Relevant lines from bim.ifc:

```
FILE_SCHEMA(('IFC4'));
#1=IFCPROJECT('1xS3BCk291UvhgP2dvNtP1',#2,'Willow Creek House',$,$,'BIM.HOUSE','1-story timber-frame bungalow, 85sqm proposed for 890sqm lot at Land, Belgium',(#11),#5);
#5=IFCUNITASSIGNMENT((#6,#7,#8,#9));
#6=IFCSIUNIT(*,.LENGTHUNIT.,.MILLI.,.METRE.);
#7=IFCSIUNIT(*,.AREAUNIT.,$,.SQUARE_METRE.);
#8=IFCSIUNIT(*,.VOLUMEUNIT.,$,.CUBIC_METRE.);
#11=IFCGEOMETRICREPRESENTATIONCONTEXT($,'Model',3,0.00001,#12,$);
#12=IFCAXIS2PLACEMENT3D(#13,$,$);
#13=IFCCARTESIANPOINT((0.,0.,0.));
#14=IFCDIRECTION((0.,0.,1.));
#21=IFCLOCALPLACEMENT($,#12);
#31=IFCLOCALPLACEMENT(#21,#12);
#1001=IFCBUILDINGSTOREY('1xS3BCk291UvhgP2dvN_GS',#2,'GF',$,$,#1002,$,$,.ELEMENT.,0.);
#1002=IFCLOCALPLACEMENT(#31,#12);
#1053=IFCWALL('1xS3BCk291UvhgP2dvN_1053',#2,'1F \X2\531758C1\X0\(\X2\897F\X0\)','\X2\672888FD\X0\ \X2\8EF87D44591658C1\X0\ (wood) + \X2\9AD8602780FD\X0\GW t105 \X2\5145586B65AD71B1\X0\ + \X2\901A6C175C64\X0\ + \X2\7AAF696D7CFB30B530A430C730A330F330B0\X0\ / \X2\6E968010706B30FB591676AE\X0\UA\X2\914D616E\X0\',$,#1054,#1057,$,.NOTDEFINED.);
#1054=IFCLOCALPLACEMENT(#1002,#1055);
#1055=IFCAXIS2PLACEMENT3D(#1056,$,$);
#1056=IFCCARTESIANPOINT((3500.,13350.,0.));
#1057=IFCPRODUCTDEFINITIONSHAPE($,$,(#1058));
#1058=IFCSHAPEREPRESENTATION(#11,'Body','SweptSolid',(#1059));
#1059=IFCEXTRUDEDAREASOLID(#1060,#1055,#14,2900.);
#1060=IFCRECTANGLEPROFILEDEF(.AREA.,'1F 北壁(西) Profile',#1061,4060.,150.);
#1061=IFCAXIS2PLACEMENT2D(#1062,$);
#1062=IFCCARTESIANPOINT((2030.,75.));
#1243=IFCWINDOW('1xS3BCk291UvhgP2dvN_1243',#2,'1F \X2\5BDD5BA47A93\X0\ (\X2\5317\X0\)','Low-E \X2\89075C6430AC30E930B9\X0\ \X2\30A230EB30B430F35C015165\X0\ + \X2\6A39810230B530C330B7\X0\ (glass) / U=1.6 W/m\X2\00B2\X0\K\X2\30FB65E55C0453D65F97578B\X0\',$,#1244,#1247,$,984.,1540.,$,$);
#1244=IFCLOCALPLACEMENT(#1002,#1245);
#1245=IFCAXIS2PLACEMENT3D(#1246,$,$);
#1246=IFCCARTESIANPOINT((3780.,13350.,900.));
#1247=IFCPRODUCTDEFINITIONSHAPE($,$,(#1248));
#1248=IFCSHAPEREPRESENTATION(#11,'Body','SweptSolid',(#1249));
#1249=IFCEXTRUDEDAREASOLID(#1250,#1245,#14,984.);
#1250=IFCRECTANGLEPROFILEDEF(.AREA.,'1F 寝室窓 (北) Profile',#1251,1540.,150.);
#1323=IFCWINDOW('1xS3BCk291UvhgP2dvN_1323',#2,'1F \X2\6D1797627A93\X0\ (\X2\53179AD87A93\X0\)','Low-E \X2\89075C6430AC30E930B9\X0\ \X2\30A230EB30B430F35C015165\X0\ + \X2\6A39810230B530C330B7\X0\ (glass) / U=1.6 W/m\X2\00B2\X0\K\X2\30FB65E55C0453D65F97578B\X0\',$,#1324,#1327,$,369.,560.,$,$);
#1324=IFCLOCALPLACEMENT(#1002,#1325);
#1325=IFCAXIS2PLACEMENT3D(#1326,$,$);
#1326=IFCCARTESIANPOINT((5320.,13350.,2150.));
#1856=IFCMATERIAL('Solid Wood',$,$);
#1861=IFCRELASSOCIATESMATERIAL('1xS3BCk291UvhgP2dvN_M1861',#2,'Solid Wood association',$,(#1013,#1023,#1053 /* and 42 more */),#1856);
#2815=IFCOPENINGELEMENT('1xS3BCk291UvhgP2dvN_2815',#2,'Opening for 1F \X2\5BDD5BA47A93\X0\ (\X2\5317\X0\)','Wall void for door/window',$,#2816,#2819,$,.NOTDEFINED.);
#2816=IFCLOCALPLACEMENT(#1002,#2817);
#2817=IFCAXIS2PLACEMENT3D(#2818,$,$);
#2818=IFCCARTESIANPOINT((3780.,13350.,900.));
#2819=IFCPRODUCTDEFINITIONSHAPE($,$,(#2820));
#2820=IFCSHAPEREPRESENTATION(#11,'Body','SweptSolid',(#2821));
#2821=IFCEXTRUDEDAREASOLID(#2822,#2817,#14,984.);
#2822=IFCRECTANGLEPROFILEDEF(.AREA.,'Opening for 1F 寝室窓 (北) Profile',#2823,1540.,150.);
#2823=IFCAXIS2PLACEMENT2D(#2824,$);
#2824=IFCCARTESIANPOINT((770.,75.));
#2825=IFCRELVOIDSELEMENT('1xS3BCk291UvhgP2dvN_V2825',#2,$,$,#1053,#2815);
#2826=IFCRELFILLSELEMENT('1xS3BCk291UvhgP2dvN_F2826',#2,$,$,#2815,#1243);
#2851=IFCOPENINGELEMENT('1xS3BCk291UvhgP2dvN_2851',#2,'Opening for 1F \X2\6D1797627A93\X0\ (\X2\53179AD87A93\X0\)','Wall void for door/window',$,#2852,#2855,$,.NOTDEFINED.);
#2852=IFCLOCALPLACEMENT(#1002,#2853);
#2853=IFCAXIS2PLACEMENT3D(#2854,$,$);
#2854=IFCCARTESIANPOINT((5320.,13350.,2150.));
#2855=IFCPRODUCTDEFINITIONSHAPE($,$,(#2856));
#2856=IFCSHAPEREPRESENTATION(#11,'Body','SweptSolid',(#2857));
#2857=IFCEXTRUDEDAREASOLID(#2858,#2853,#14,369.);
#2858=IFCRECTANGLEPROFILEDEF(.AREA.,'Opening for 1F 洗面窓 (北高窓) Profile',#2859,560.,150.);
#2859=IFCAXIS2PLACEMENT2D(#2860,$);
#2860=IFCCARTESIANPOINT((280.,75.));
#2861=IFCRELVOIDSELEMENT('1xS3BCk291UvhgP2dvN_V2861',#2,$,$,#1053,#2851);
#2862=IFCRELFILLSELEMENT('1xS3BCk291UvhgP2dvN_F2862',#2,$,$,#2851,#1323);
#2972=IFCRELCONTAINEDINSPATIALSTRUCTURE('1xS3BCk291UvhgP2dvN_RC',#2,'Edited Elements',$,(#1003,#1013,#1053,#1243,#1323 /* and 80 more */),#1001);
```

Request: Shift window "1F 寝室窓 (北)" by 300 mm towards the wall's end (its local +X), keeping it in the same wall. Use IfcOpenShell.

```python
import ifcopenshell
import ifcopenshell.api.geometry
import ifcopenshell.util.placement

model = ifcopenshell.open("bim.ifc")

window = model.by_guid("1xS3BCk291UvhgP2dvN_1243")
opening = window.FillsVoids[0].RelatingOpeningElement
wall = opening.VoidsElements[0].RelatingBuildingElement

wall_matrix = ifcopenshell.util.placement.get_local_placement(wall.ObjectPlacement)
shift = wall_matrix[:3, 0] * 300.0
before = ifcopenshell.util.placement.get_local_placement(window.ObjectPlacement)[:3, 3].copy()

# The window is not placed relative to its opening, so move both.
for product in (opening, window):
    matrix = ifcopenshell.util.placement.get_local_placement(product.ObjectPlacement)
    matrix[:3, 3] += shift
    ifcopenshell.api.geometry.edit_object_placement(model, product=product, matrix=matrix, is_si=False)

after = ifcopenshell.util.placement.get_local_placement(window.ObjectPlacement)[:3, 3]
print("window moved by", (after - before).round(3) + 0.0)

model.write("bim-out.ifc")
```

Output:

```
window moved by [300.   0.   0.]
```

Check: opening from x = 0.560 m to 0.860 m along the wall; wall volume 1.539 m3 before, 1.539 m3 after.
